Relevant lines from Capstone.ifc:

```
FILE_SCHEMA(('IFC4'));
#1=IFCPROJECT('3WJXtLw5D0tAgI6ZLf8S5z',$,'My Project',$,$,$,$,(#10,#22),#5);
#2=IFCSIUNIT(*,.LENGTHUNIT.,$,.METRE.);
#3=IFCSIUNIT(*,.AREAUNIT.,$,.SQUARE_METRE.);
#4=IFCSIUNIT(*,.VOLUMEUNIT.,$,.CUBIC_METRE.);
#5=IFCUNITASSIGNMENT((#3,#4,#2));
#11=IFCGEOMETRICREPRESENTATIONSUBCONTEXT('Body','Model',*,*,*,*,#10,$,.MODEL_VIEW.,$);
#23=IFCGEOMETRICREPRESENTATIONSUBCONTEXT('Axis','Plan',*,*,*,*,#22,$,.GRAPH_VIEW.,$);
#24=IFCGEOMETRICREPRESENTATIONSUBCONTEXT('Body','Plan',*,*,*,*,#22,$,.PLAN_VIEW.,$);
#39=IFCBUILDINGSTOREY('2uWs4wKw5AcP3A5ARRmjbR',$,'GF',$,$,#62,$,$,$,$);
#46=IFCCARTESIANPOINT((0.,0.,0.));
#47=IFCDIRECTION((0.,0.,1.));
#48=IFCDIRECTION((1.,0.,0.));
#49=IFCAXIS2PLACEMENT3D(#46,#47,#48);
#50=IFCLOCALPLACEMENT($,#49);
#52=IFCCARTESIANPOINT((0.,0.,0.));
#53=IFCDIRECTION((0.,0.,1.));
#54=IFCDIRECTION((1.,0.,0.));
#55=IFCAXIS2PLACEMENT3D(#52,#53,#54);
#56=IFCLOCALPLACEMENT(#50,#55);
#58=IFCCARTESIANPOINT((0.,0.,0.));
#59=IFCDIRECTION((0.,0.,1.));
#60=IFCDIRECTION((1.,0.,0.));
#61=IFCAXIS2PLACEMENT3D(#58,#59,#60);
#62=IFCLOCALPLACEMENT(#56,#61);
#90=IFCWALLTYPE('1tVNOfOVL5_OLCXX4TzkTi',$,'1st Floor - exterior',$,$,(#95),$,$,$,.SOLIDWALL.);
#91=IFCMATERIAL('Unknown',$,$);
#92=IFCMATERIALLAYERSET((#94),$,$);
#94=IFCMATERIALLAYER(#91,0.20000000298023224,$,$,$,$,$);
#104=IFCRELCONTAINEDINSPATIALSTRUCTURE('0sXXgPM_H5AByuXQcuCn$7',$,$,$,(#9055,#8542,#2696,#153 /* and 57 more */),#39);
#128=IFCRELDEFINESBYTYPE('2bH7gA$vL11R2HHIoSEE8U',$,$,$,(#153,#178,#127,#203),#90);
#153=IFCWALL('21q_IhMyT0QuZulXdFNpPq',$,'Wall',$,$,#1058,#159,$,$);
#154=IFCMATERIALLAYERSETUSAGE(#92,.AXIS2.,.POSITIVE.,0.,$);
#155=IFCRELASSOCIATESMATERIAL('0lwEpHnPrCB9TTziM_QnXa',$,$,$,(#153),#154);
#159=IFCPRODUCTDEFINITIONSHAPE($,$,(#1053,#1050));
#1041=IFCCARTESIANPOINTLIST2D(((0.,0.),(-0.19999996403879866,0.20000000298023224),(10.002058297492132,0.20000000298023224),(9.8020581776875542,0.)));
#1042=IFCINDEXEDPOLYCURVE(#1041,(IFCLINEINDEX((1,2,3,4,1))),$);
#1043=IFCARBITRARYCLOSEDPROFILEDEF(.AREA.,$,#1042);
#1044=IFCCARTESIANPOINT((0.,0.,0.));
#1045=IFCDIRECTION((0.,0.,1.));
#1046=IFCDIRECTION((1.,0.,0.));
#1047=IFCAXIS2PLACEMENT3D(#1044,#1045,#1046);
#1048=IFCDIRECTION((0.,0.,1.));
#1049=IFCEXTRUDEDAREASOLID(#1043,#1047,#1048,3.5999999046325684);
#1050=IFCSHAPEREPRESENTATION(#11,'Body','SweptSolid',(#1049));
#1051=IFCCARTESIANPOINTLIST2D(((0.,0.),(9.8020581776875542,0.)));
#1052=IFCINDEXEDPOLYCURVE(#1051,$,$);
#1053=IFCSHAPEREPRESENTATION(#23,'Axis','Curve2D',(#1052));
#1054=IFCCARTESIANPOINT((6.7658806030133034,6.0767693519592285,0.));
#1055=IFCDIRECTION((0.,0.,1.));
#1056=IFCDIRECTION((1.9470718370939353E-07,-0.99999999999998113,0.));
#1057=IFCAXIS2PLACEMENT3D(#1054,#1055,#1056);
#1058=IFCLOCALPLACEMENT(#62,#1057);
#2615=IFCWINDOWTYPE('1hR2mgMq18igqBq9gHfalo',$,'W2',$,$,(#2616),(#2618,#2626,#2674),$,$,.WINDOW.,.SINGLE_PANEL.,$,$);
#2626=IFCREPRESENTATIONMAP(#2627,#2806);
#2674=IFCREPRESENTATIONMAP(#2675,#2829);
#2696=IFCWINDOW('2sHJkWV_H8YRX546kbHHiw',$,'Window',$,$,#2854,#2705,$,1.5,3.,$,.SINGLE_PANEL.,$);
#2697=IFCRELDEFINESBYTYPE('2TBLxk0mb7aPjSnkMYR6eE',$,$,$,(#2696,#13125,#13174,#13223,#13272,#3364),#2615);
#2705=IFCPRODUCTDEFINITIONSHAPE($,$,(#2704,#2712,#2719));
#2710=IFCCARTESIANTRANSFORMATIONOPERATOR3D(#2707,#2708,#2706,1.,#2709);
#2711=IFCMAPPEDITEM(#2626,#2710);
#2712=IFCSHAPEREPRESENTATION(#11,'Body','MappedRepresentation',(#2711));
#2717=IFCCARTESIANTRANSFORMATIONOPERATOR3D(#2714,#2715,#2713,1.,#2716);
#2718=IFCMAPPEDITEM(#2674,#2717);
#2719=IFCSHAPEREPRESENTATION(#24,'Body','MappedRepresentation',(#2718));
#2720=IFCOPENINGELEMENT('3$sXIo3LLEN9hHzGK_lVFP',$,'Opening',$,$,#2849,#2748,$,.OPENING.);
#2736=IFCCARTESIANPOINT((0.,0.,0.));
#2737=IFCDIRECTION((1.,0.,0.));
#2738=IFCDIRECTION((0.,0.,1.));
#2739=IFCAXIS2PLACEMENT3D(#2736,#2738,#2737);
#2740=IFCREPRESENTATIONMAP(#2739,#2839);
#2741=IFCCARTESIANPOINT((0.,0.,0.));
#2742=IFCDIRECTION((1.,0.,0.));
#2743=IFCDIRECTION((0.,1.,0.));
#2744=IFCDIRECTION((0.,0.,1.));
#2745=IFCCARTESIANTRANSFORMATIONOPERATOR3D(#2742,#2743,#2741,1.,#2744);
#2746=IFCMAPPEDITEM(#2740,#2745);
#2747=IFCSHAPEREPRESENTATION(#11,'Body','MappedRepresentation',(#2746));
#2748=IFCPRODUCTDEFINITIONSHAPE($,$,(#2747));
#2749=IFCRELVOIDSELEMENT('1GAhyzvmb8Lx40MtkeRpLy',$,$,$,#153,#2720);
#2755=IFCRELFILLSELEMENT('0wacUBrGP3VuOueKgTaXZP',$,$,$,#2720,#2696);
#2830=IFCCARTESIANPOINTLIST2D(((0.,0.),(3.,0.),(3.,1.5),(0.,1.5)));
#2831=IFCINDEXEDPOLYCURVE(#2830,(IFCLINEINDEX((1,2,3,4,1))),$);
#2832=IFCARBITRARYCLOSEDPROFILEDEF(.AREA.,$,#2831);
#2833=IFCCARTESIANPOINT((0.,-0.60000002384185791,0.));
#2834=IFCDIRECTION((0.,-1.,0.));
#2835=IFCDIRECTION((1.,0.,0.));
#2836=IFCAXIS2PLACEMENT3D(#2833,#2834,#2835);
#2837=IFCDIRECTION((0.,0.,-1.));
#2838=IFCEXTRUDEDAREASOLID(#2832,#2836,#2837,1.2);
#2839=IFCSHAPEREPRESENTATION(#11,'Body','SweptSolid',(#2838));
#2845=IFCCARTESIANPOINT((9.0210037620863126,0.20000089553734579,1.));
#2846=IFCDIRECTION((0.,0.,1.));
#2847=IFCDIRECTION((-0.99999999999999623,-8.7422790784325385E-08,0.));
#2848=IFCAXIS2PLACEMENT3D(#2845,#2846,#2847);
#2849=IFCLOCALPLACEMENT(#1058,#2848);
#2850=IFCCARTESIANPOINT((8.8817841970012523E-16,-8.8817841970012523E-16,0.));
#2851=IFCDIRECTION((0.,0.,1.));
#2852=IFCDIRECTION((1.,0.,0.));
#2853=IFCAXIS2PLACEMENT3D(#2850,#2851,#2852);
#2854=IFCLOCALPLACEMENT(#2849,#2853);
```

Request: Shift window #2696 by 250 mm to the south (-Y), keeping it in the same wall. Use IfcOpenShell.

```python
import ifcopenshell
import ifcopenshell.api.geometry
import ifcopenshell.util.placement

model = ifcopenshell.open("Capstone.ifc")

window = model.by_guid("2sHJkWV_H8YRX546kbHHiw")
opening = window.FillsVoids[0].RelatingOpeningElement
wall = opening.VoidsElements[0].RelatingBuildingElement

wall_matrix = ifcopenshell.util.placement.get_local_placement(wall.ObjectPlacement)
shift = wall_matrix[:3, 0] * 0.25
before = ifcopenshell.util.placement.get_local_placement(window.ObjectPlacement)[:3, 3].copy()

# The window is placed relative to its opening, so it follows when the opening moves.
matrix = ifcopenshell.util.placement.get_local_placement(opening.ObjectPlacement)
matrix[:3, 3] += shift
ifcopenshell.api.geometry.edit_object_placement(
    model, product=opening, matrix=matrix, is_si=False, should_transform_children=True
)

after = ifcopenshell.util.placement.get_local_placement(window.ObjectPlacement)[:3, 3]
print("window moved by", (after - before).round(3) + 0.0)

model.write("Capstone_rev.ifc")
```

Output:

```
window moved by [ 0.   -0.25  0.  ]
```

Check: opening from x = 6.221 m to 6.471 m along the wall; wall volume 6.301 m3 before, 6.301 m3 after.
